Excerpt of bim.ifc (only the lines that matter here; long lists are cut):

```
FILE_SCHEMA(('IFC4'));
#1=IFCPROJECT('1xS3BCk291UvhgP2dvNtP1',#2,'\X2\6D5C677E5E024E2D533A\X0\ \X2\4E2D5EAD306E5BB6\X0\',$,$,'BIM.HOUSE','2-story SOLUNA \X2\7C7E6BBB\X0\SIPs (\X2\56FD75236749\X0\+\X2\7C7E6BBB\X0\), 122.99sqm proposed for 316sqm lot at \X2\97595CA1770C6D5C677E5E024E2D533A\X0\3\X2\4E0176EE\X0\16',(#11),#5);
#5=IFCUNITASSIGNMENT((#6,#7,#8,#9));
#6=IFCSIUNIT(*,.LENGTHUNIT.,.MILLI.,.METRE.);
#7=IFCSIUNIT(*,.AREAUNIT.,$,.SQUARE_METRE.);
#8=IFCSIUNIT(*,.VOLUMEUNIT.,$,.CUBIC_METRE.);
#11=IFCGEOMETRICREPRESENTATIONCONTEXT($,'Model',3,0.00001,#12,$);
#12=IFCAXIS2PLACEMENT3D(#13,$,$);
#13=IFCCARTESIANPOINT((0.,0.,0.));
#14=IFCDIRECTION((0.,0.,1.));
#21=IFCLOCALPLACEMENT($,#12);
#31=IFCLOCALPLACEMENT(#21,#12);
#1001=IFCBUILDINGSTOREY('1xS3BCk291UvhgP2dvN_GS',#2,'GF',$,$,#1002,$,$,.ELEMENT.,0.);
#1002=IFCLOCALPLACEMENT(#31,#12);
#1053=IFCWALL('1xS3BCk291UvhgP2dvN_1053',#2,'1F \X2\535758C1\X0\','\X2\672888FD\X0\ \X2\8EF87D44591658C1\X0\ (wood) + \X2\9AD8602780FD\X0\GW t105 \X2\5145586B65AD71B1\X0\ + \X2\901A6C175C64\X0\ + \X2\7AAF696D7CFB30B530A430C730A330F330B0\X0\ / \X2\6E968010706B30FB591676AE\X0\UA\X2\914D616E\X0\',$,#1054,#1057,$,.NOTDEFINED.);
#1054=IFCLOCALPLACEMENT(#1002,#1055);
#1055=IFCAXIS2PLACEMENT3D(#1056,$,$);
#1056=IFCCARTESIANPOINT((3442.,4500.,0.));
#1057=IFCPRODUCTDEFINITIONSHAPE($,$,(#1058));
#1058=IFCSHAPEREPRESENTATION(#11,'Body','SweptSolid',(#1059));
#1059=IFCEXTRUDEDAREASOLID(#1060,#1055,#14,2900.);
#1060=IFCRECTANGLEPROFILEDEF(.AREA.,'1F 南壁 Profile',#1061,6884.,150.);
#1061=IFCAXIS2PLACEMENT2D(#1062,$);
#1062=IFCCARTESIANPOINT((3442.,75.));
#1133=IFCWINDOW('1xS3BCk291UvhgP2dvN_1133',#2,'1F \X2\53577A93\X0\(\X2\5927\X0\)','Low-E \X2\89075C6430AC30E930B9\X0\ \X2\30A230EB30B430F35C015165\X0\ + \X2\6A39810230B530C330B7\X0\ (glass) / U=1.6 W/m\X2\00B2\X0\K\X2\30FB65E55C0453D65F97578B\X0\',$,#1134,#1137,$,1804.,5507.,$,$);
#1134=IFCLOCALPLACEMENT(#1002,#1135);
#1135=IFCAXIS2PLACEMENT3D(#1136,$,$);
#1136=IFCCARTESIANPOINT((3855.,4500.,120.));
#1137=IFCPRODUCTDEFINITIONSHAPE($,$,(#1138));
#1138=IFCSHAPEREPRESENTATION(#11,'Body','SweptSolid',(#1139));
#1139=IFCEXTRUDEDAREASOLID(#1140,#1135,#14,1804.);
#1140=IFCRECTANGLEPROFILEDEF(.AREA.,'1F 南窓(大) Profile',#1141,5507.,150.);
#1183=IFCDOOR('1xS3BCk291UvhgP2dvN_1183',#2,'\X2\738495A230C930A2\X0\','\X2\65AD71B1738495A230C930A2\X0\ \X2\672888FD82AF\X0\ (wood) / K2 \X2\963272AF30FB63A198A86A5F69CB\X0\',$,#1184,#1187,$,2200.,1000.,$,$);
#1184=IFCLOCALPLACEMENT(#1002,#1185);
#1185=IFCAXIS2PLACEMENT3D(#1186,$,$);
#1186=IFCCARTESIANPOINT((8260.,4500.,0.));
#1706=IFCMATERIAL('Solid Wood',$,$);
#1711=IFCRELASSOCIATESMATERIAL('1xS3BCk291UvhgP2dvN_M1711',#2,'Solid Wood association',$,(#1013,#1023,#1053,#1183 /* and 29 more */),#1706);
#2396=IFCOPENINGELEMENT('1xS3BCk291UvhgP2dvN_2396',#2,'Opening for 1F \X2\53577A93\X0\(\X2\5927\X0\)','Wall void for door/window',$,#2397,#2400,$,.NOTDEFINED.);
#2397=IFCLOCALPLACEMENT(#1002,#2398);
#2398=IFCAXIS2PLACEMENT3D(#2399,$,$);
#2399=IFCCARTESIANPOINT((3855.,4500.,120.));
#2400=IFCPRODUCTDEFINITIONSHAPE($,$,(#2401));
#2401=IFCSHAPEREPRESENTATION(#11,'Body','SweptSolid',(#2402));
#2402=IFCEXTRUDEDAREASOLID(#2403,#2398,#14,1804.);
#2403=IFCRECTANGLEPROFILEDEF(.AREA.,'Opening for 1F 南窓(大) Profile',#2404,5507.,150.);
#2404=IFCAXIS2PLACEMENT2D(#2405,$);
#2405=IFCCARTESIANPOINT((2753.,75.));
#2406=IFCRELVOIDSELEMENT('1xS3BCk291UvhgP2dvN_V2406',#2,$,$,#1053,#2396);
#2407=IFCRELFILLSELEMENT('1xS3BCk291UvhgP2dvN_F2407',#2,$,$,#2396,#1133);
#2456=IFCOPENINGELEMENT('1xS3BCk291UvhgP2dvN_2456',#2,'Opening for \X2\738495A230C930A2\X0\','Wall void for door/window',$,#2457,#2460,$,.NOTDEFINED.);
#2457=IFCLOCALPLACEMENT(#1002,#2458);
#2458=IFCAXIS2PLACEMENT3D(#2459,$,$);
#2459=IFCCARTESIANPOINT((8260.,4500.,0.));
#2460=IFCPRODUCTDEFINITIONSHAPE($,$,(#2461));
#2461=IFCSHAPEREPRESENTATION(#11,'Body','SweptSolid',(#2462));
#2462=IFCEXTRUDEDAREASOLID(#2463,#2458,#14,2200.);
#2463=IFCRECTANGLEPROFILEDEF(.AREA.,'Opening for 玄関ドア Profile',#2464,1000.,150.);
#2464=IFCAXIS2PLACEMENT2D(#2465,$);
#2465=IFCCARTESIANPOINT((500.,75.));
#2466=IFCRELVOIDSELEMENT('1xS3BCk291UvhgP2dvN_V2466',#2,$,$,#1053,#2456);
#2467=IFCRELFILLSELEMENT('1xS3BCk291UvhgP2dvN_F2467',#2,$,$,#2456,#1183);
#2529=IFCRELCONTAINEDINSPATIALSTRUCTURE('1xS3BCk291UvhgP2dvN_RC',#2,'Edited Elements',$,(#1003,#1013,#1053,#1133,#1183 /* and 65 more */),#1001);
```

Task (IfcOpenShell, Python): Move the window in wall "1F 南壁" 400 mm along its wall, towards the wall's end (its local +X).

```python
import ifcopenshell
import ifcopenshell.api.geometry
import ifcopenshell.util.placement
import ifcopenshell.util.unit

model = ifcopenshell.open("bim.ifc")
unit_scale = ifcopenshell.util.unit.calculate_unit_scale(model)

window = model.by_guid("1xS3BCk291UvhgP2dvN_1133")
opening = window.FillsVoids[0].RelatingOpeningElement
wall = opening.VoidsElements[0].RelatingBuildingElement

wall_matrix = ifcopenshell.util.placement.get_local_placement(wall.ObjectPlacement)
shift = wall_matrix[:3, 0] * 0.4 / unit_scale
before = ifcopenshell.util.placement.get_local_placement(window.ObjectPlacement)[:3, 3].copy()

# The window is not placed relative to its opening, so move both.
for product in (opening, window):
    matrix = ifcopenshell.util.placement.get_local_placement(product.ObjectPlacement)
    matrix[:3, 3] += shift
    ifcopenshell.api.geometry.edit_object_placement(model, product=product, matrix=matrix, is_si=False)

after = ifcopenshell.util.placement.get_local_placement(window.ObjectPlacement)[:3, 3]
print("window moved by", (after - before).round(3) + 0.0)

model.write("bim-out.ifc")
```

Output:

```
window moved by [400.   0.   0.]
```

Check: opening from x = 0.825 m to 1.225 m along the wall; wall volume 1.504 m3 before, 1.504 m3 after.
